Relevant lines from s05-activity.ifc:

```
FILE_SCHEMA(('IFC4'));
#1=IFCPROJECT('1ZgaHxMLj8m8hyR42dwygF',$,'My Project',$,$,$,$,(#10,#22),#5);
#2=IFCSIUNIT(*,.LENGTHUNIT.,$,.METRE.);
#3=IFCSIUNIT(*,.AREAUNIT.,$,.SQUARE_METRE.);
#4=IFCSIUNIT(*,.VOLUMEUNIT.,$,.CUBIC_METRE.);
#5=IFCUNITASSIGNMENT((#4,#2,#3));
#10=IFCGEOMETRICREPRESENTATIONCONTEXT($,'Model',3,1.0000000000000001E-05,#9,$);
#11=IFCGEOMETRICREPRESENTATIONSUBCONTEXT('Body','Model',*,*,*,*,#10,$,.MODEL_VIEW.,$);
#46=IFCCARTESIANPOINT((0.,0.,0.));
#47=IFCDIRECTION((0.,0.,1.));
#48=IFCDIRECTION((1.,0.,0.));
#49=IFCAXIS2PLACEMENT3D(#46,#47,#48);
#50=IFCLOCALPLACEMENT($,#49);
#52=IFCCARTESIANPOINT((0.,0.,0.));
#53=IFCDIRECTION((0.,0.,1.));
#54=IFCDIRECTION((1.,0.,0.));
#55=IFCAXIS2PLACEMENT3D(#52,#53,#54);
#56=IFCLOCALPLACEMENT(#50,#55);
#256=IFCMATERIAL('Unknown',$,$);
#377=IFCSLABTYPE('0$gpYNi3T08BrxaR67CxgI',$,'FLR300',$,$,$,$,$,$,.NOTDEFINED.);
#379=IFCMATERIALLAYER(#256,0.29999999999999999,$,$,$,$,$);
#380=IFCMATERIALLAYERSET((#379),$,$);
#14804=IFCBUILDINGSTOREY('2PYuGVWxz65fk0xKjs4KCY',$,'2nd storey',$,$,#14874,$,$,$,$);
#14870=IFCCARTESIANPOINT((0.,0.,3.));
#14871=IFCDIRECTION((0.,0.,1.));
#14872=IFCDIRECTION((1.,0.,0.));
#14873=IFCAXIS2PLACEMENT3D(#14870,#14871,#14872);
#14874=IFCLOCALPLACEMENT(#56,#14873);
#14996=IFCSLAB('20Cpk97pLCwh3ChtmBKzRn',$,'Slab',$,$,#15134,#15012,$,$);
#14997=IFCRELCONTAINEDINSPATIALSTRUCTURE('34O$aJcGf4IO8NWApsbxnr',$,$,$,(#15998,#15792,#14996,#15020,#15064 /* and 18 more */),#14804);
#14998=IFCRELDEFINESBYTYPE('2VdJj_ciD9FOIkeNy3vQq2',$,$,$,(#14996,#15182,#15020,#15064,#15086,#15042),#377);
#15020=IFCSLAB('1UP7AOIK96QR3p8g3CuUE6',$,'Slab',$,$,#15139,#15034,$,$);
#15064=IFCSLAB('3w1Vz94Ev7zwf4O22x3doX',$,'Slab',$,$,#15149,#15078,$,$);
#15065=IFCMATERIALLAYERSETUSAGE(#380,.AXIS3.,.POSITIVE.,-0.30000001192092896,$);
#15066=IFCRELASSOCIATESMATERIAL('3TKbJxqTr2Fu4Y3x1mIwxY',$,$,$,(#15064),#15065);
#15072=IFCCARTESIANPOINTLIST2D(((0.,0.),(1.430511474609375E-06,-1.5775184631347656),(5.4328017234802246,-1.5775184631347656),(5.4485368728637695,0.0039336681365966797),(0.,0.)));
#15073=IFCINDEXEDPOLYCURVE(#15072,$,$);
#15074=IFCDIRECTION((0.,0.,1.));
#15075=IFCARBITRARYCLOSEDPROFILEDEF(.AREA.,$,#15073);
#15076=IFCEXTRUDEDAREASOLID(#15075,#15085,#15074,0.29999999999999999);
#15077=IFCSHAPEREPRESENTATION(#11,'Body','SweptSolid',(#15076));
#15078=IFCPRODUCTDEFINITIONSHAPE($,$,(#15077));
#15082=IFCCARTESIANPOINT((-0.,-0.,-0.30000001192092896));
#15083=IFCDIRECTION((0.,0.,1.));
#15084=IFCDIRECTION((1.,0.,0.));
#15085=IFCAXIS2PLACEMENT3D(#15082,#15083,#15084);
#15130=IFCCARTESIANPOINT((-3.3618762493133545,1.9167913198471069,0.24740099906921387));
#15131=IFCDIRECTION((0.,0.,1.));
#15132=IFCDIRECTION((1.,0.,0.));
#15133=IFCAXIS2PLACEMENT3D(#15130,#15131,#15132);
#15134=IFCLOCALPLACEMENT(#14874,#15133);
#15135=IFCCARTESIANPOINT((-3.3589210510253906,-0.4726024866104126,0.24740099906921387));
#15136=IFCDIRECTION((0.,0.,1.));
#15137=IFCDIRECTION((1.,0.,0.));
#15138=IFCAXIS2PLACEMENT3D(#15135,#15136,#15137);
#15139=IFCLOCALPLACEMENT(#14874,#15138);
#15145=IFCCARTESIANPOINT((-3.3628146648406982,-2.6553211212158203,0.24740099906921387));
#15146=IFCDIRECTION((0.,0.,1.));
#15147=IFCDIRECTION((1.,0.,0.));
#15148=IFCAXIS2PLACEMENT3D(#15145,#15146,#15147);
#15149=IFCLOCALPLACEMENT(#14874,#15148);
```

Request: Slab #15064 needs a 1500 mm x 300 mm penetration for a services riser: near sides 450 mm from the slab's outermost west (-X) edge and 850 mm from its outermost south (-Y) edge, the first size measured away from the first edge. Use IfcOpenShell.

```python
import numpy as np
import ifcopenshell
import ifcopenshell.api.feature
import ifcopenshell.api.geometry
import ifcopenshell.api.root
import ifcopenshell.geom
import ifcopenshell.util.placement
import ifcopenshell.util.representation
import ifcopenshell.util.shape
import ifcopenshell.util.unit

model = ifcopenshell.open("s05-activity.ifc")
unit_scale = ifcopenshell.util.unit.calculate_unit_scale(model)
settings = ifcopenshell.geom.settings()


def volume(element):
    """Net volume in cubic metres, openings subtracted."""
    shape = ifcopenshell.geom.create_shape(settings, element)
    return ifcopenshell.util.shape.get_volume(shape.geometry)


slab = model.by_id(15064)
before = volume(slab)

# Extent in the slab's own axes, in metres. The edges named are its -X and -Y sides.
slab_shape = ifcopenshell.geom.create_shape(settings, slab)
vertices = ifcopenshell.util.shape.get_vertices(slab_shape.geometry)
x_min, y_min, bottom = vertices.min(axis=0)
top = vertices[:, 2].max()

opening = ifcopenshell.api.root.create_entity(model, ifc_class="IfcOpeningElement", name="Services riser opening", predefined_type="OPENING")
context = ifcopenshell.util.representation.get_context(model, "Model", "Body", "MODEL_VIEW")
width, depth = 1.5, 0.3
outline = [(0.0, 0.0), (width, 0.0), (width, depth), (0.0, depth), (0.0, 0.0)]
# Overshoot both faces by 50 mm so the cut is clean.
shape = ifcopenshell.api.geometry.add_slab_representation(
    model, context=context, depth=top - bottom + 0.1, polyline=outline
)
ifcopenshell.api.geometry.assign_representation(model, product=opening, representation=shape)

matrix = ifcopenshell.util.placement.get_local_placement(slab.ObjectPlacement)
matrix[:, 3] = matrix @ np.append(np.array([x_min + 0.45, y_min + 0.85, bottom - 0.05]) / unit_scale, 1.0)
ifcopenshell.api.geometry.edit_object_placement(model, product=opening, matrix=matrix, is_si=False)
ifcopenshell.api.feature.add_feature(model, feature=opening, element=slab)

after = volume(slab)

print(f"slab volume {before:.3f} -> {after:.3f} m3")

model.write("s05-activity_rev.ifc")
```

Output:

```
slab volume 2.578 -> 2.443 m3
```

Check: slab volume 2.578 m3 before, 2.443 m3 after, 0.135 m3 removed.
